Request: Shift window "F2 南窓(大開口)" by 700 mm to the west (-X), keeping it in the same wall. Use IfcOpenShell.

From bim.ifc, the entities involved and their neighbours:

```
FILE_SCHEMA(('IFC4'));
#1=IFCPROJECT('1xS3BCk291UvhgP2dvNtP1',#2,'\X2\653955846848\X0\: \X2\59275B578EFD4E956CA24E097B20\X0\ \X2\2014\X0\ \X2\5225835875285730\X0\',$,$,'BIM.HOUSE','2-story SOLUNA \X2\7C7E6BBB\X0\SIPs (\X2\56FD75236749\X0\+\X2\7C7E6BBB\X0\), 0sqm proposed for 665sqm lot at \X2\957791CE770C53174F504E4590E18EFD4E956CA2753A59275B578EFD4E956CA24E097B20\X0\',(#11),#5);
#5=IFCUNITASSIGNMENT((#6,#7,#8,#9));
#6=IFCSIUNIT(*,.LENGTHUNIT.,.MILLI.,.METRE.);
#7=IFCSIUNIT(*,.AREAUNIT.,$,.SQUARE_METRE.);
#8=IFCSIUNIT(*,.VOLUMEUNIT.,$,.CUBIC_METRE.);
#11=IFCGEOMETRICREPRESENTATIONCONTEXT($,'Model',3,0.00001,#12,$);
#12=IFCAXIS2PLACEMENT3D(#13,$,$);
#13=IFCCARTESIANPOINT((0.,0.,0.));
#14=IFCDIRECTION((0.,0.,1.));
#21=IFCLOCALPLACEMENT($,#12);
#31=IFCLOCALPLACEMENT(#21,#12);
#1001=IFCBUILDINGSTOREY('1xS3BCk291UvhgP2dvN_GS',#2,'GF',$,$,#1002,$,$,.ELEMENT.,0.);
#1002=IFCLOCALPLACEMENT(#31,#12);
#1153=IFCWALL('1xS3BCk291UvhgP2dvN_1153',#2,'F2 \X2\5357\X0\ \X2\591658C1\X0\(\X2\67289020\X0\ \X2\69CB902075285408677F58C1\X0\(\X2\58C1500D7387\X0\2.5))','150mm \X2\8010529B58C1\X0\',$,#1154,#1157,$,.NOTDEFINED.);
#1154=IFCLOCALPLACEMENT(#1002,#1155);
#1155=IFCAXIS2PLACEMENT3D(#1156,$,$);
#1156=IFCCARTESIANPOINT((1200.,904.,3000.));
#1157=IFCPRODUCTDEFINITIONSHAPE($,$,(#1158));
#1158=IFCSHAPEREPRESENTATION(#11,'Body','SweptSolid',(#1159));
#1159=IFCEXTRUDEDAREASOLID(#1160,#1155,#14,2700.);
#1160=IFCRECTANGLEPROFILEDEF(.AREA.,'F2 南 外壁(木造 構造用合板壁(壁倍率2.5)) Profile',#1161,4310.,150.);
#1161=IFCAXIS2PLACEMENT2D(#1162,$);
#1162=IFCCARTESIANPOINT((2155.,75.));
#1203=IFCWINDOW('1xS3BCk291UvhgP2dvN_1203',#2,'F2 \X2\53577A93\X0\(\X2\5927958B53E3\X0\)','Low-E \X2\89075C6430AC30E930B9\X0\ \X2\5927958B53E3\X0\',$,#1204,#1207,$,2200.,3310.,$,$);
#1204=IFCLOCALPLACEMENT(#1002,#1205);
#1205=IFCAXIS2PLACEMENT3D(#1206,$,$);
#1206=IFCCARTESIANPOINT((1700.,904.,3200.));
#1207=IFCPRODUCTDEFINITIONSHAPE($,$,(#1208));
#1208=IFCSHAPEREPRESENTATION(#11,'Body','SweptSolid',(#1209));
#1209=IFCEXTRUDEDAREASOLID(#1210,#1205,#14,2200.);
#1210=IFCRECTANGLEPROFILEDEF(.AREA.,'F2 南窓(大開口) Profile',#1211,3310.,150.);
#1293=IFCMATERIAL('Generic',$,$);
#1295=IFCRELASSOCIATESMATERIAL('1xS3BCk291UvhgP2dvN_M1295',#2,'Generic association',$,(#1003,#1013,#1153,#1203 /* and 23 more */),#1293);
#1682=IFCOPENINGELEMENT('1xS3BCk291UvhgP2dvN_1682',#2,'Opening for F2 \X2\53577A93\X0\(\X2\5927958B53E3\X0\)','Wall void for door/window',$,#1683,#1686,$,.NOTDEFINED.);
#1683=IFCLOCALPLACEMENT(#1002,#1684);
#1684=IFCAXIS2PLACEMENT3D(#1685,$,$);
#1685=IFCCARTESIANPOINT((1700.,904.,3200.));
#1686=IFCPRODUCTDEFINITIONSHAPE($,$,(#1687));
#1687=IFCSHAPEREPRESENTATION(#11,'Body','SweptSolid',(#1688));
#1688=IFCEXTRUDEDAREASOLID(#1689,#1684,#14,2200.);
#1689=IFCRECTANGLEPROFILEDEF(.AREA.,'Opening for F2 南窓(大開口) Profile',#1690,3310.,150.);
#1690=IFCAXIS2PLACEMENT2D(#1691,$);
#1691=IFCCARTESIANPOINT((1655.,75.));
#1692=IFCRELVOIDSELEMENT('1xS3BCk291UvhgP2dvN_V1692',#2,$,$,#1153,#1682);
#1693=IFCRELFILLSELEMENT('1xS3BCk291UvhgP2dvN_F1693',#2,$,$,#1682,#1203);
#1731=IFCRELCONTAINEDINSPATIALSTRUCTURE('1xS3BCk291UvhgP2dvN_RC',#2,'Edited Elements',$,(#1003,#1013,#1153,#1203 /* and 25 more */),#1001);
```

```python
import ifcopenshell
import ifcopenshell.api.geometry
import ifcopenshell.util.placement

model = ifcopenshell.open("bim.ifc")

window = model.by_id(1203)
opening = window.FillsVoids[0].RelatingOpeningElement
wall = opening.VoidsElements[0].RelatingBuildingElement

wall_matrix = ifcopenshell.util.placement.get_local_placement(wall.ObjectPlacement)
shift = wall_matrix[:3, 0] * -700.0
before = ifcopenshell.util.placement.get_local_placement(window.ObjectPlacement)[:3, 3].copy()

# The window is not placed relative to its opening, so move both.
for product in (opening, window):
    matrix = ifcopenshell.util.placement.get_local_placement(product.ObjectPlacement)
    matrix[:3, 3] += shift
    ifcopenshell.api.geometry.edit_object_placement(model, product=product, matrix=matrix, is_si=False)

after = ifcopenshell.util.placement.get_local_placement(window.ObjectPlacement)[:3, 3]
print("window moved by", (after - before).round(3) + 0.0)

model.write("bim_updated.ifc")
```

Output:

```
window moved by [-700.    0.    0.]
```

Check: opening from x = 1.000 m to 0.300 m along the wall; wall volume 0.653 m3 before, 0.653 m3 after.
